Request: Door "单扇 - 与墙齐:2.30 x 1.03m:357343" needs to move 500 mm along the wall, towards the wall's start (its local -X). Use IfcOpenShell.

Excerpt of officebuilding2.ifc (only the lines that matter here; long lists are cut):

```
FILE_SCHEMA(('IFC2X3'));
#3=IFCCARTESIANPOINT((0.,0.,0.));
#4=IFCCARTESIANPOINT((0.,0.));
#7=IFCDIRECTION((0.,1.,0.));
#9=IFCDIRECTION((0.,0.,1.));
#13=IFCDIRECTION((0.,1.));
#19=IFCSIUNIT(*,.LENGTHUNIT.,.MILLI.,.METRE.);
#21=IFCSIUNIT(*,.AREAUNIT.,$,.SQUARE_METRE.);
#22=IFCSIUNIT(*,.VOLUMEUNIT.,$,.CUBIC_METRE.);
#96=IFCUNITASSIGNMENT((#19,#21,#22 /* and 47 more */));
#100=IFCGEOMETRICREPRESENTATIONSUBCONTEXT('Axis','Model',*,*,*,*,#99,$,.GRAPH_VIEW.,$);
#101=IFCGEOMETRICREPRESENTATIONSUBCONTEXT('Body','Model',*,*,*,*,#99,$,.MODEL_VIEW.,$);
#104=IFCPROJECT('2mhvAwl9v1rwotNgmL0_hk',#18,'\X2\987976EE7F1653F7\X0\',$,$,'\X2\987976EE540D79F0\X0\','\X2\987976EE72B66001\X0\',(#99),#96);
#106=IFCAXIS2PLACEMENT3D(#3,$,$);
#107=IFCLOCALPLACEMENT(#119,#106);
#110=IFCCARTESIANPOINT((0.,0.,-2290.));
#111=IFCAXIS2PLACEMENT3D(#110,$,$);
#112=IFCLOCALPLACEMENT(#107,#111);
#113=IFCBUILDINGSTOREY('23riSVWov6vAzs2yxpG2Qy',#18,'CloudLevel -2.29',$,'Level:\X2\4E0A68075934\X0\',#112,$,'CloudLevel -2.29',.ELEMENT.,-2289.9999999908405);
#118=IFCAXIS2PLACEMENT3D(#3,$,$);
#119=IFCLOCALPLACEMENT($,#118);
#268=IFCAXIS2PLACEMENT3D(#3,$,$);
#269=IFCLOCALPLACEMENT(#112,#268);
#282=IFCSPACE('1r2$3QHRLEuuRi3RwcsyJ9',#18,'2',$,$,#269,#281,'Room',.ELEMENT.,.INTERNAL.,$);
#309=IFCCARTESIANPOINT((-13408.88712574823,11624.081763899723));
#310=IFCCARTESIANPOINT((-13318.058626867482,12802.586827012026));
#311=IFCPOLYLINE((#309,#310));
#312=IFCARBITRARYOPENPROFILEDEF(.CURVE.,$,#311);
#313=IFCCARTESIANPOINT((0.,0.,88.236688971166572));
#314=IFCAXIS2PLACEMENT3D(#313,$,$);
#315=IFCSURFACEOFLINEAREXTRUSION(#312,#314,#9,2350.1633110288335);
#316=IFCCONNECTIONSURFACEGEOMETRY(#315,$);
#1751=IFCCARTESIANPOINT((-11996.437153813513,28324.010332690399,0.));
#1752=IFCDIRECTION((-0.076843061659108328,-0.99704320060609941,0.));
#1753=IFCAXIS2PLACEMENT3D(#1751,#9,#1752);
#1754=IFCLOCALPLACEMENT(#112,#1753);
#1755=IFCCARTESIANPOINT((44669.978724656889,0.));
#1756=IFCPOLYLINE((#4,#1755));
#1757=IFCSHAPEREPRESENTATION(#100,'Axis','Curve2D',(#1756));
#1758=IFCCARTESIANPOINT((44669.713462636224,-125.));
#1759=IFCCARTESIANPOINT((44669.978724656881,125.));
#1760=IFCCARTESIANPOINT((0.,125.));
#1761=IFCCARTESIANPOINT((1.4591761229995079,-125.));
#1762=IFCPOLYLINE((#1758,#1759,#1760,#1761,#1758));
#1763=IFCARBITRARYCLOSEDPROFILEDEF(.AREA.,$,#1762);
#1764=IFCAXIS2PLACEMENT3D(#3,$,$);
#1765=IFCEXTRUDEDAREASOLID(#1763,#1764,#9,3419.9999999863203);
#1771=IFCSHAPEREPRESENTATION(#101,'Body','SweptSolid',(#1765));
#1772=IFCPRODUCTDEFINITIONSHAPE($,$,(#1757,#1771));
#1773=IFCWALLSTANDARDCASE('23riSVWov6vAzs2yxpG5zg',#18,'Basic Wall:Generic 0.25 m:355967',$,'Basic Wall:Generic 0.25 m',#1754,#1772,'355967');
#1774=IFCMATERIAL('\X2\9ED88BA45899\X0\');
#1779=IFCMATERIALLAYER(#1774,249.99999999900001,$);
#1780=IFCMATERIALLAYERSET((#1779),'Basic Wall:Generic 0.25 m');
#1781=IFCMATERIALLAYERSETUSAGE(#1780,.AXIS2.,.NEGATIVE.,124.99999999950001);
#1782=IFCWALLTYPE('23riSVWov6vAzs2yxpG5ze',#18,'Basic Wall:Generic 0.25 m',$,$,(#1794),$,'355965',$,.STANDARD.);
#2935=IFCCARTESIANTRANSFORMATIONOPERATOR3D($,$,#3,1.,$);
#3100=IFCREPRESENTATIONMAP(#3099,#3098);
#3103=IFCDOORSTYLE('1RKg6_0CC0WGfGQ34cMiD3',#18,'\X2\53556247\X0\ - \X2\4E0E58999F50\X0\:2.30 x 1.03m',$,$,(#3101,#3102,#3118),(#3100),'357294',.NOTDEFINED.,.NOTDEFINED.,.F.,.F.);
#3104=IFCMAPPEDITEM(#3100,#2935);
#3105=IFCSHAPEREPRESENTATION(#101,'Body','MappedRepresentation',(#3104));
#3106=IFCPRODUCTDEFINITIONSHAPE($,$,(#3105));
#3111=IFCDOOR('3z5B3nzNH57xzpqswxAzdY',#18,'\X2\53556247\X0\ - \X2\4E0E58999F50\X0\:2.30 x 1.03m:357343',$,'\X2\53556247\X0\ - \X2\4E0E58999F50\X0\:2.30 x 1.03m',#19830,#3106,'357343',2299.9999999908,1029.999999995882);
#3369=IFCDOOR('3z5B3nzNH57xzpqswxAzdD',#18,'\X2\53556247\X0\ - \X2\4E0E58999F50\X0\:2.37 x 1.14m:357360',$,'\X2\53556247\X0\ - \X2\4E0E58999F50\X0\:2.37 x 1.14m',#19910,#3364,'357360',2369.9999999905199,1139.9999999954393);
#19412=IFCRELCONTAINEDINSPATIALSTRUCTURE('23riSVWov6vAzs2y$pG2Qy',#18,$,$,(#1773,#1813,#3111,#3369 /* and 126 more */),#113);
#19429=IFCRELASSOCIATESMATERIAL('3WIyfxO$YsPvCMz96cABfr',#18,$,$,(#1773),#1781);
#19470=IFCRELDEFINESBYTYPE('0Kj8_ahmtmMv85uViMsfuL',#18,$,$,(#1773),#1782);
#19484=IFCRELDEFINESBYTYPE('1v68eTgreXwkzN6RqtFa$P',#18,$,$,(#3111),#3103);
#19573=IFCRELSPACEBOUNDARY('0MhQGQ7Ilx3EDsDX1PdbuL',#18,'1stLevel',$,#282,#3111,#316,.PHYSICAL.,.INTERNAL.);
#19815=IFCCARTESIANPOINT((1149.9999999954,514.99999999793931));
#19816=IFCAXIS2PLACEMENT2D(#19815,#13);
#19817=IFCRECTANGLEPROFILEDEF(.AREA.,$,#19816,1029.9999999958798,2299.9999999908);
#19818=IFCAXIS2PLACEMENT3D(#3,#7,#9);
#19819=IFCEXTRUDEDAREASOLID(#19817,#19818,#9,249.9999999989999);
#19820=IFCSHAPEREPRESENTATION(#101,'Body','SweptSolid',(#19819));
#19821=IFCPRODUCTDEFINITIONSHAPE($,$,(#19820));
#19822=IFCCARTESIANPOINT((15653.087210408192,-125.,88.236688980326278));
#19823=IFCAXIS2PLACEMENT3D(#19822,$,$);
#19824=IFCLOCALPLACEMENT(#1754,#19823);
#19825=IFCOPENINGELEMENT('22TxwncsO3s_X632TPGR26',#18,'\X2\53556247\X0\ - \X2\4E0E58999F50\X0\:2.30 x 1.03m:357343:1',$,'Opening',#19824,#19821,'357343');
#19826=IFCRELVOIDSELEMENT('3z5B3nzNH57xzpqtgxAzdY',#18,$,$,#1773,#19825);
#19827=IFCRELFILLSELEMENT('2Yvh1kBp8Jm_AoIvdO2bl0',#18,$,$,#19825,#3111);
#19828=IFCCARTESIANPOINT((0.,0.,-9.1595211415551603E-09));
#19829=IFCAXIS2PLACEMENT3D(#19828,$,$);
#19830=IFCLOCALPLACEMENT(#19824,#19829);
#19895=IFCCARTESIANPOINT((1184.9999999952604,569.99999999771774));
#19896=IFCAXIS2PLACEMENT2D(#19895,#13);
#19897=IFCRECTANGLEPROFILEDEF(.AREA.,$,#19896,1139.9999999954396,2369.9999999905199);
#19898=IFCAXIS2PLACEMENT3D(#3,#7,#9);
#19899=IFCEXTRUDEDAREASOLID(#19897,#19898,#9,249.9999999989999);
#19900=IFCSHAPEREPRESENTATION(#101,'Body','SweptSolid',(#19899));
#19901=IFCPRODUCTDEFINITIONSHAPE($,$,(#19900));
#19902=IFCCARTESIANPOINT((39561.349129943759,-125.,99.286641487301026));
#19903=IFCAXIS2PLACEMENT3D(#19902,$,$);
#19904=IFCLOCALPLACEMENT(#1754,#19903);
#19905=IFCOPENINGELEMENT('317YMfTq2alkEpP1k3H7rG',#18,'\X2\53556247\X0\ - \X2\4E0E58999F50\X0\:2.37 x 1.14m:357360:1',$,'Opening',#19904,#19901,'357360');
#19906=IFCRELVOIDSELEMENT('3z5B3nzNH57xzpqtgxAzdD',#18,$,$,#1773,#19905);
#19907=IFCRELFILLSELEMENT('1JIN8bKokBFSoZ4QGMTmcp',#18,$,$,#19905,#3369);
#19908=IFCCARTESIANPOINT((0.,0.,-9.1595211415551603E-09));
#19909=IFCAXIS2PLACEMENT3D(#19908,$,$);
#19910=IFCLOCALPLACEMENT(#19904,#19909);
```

```python
import numpy as np
import ifcopenshell
import ifcopenshell.api.geometry
import ifcopenshell.util.placement
import ifcopenshell.util.unit

model = ifcopenshell.open("officebuilding2.ifc")
unit_scale = ifcopenshell.util.unit.calculate_unit_scale(model)

door = model.by_id(3111)
opening = door.FillsVoids[0].RelatingOpeningElement
wall = opening.VoidsElements[0].RelatingBuildingElement

wall_matrix = ifcopenshell.util.placement.get_local_placement(wall.ObjectPlacement)
shift = wall_matrix[:3, 0] * -0.5 / unit_scale
before = ifcopenshell.util.placement.get_local_placement(door.ObjectPlacement)[:3, 3].copy()

# The door is placed relative to its opening, so it follows when the opening moves.
matrix = ifcopenshell.util.placement.get_local_placement(opening.ObjectPlacement)
matrix[:3, 3] += shift
ifcopenshell.api.geometry.edit_object_placement(
    model, product=opening, matrix=matrix, is_si=False, should_transform_children=True
)

# Space boundary surfaces are stored in each space's coordinates; move them too.
for rel in door.ProvidesBoundaries:
    if not rel.ConnectionGeometry:
        continue
    surface = rel.ConnectionGeometry.SurfaceOnRelatingElement
    space_matrix = ifcopenshell.util.placement.get_local_placement(rel.RelatingSpace.ObjectPlacement)
    point = np.array(surface.Position.Location.Coordinates) + space_matrix[:3, :3].T @ shift
    surface.Position = model.createIfcAxis2Placement3D(
        model.createIfcCartesianPoint(point.tolist()), surface.Position.Axis, surface.Position.RefDirection
    )

after = ifcopenshell.util.placement.get_local_placement(door.ObjectPlacement)[:3, 3]
print("door moved by", (after - before).round(3) + 0.0)

model.write("officebuilding2_edited.ifc")
```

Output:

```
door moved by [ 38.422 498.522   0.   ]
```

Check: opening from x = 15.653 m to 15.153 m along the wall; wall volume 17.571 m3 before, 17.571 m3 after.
